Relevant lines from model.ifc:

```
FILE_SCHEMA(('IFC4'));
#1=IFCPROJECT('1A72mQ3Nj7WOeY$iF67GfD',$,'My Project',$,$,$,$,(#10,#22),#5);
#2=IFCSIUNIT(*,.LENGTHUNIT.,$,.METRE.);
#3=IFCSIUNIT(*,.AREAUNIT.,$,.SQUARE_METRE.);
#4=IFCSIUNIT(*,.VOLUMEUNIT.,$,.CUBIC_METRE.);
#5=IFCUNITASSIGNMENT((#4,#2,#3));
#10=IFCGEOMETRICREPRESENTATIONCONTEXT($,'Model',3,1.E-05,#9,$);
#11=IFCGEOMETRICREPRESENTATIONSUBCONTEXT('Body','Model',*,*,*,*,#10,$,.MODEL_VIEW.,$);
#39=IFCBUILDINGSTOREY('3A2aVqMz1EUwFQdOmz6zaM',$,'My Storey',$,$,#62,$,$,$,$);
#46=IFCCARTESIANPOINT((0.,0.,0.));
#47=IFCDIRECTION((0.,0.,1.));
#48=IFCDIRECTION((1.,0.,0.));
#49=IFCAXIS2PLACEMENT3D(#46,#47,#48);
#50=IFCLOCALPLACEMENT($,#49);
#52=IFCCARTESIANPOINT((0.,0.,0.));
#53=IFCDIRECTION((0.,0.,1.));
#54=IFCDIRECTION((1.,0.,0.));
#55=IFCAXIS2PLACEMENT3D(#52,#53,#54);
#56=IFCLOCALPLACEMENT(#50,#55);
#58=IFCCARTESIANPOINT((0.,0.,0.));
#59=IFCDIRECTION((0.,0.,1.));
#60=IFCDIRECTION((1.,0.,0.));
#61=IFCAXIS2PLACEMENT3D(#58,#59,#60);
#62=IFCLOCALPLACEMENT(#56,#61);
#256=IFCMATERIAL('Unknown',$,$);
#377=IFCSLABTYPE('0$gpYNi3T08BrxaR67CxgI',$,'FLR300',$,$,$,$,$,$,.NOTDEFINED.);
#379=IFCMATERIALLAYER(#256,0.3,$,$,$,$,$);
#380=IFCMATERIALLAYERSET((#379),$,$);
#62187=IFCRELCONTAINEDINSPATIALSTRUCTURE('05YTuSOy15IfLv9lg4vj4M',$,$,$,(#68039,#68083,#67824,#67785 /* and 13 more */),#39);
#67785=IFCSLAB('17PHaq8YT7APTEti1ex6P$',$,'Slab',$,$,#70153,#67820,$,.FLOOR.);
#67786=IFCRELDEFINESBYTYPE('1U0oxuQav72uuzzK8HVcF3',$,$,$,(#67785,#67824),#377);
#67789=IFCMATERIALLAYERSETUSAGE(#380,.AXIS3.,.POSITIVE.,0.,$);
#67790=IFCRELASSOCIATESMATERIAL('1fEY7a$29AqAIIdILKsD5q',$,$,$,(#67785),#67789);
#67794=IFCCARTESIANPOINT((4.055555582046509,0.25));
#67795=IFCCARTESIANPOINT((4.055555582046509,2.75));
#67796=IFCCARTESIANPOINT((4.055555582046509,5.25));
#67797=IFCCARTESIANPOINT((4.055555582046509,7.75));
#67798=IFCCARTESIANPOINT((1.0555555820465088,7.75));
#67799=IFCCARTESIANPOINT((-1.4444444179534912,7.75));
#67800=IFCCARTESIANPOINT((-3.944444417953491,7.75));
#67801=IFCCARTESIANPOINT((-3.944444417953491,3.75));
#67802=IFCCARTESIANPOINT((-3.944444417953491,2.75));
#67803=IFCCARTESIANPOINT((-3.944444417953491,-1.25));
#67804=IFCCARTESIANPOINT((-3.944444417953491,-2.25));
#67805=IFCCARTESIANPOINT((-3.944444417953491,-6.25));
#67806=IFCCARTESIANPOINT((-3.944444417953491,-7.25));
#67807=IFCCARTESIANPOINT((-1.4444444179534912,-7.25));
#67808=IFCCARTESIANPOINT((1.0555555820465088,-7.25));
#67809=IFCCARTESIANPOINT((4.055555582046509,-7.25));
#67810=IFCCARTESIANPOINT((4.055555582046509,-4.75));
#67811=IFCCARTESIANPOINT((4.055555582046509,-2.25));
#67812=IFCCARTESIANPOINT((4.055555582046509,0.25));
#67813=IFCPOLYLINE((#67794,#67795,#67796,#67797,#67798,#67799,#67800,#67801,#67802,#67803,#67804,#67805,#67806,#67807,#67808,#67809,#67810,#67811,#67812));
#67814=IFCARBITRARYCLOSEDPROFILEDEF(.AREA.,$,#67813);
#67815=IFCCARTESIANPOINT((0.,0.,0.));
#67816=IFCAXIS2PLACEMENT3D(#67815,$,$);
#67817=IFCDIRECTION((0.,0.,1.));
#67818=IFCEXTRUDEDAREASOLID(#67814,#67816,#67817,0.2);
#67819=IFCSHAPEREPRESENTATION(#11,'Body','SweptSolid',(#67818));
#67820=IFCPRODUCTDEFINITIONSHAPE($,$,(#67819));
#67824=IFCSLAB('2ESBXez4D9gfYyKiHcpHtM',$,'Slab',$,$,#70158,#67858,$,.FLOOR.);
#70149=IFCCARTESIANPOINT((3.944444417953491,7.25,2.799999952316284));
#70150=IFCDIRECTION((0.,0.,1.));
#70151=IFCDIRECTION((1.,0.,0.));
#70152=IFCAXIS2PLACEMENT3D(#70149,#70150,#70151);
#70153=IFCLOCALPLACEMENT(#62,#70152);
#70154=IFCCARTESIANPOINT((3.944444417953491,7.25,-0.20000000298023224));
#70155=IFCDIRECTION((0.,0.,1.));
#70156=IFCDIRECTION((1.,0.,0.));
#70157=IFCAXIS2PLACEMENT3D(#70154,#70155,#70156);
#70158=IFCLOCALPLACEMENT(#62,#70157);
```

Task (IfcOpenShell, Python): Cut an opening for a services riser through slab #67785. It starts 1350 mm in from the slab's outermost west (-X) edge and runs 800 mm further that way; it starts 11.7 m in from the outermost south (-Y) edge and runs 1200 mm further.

```python
import numpy as np
import ifcopenshell
import ifcopenshell.api.feature
import ifcopenshell.api.geometry
import ifcopenshell.api.root
import ifcopenshell.geom
import ifcopenshell.util.placement
import ifcopenshell.util.representation
import ifcopenshell.util.shape
import ifcopenshell.util.unit

model = ifcopenshell.open("model.ifc")
unit_scale = ifcopenshell.util.unit.calculate_unit_scale(model)
settings = ifcopenshell.geom.settings()


def volume(element):
    """Net volume in cubic metres, openings subtracted."""
    shape = ifcopenshell.geom.create_shape(settings, element)
    return ifcopenshell.util.shape.get_volume(shape.geometry)


slab = model.by_id(67785)
before = volume(slab)

# Extent in the slab's own axes, in metres. The edges named are its -X and -Y sides.
slab_shape = ifcopenshell.geom.create_shape(settings, slab)
vertices = ifcopenshell.util.shape.get_vertices(slab_shape.geometry)
x_min, y_min, bottom = vertices.min(axis=0)
top = vertices[:, 2].max()

opening = ifcopenshell.api.root.create_entity(model, ifc_class="IfcOpeningElement", name="Services riser opening", predefined_type="OPENING")
context = ifcopenshell.util.representation.get_context(model, "Model", "Body", "MODEL_VIEW")
width, depth = 0.8, 1.2
outline = [(0.0, 0.0), (width, 0.0), (width, depth), (0.0, depth), (0.0, 0.0)]
# Overshoot both faces by 50 mm so the cut is clean.
shape = ifcopenshell.api.geometry.add_slab_representation(
    model, context=context, depth=top - bottom + 0.1, polyline=outline
)
ifcopenshell.api.geometry.assign_representation(model, product=opening, representation=shape)

matrix = ifcopenshell.util.placement.get_local_placement(slab.ObjectPlacement)
matrix[:, 3] = matrix @ np.append(np.array([x_min + 1.35, y_min + 11.7, bottom - 0.05]) / unit_scale, 1.0)
ifcopenshell.api.geometry.edit_object_placement(model, product=opening, matrix=matrix, is_si=False)
ifcopenshell.api.feature.add_feature(model, feature=opening, element=slab)

after = volume(slab)

print(f"slab volume {before:.3f} -> {after:.3f} m3")

model.write("model_updated.ifc")
```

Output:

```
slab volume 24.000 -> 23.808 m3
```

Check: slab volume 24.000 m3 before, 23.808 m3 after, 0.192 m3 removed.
